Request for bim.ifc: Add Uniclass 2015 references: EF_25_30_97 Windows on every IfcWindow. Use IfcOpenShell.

First a look at what the model holds.

```python
import ifcopenshell

model = ifcopenshell.open("bim.ifc")
print(model.schema)
print("classifications:", [c.Name for c in model.by_type("IfcClassification")])
for ifc_class in ("IfcDoor", "IfcRoof", "IfcStair", "IfcWall", "IfcWindow"):
    print(ifc_class, len(model.by_type(ifc_class)))
```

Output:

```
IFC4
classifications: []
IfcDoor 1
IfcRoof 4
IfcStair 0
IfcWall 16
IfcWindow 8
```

```python
import ifcopenshell
import ifcopenshell.api.classification

model = ifcopenshell.open("bim.ifc")

system = ifcopenshell.api.classification.add_classification(model, classification="Uniclass 2015")

codes = {
    "IfcWindow": ("EF_25_30_97", "Windows"),
}
for ifc_class, (code, name) in codes.items():
    products = model.by_type(ifc_class)
    ifcopenshell.api.classification.add_reference(
        model, products=products, classification=system, identification=code, name=name
    )
    print(code, len(products))

model.write("bim_v2.ifc")
```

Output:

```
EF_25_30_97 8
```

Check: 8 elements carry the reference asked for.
